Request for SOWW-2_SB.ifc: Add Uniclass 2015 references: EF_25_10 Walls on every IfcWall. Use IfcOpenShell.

First a look at what the model holds.

```python
import ifcopenshell

model = ifcopenshell.open("SOWW-2_SB.ifc")
print(model.schema)
print("classifications:", [c.Name for c in model.by_type("IfcClassification")])
for ifc_class in ("IfcDoor", "IfcRoof", "IfcStair", "IfcWall", "IfcWindow"):
    print(ifc_class, len(model.by_type(ifc_class)))
```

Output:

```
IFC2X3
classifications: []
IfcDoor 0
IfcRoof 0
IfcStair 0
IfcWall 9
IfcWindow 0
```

```python
import ifcopenshell
import ifcopenshell.api.classification

model = ifcopenshell.open("SOWW-2_SB.ifc")

# IFC2X3 requires Source and Edition and has no link from the project to the system.
system = model.create_entity("IfcClassification", Source="NBS", Edition="2015", Name="Uniclass 2015")

codes = {
    "IfcWall": ("EF_25_10", "Walls"),
}
for ifc_class, (code, name) in codes.items():
    products = model.by_type(ifc_class)
    ifcopenshell.api.classification.add_reference(
        model, products=products, classification=system, identification=code, name=name
    )
    print(code, len(products))

model.write("SOWW-2_SB_v2.ifc")
```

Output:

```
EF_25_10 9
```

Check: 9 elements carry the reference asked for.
